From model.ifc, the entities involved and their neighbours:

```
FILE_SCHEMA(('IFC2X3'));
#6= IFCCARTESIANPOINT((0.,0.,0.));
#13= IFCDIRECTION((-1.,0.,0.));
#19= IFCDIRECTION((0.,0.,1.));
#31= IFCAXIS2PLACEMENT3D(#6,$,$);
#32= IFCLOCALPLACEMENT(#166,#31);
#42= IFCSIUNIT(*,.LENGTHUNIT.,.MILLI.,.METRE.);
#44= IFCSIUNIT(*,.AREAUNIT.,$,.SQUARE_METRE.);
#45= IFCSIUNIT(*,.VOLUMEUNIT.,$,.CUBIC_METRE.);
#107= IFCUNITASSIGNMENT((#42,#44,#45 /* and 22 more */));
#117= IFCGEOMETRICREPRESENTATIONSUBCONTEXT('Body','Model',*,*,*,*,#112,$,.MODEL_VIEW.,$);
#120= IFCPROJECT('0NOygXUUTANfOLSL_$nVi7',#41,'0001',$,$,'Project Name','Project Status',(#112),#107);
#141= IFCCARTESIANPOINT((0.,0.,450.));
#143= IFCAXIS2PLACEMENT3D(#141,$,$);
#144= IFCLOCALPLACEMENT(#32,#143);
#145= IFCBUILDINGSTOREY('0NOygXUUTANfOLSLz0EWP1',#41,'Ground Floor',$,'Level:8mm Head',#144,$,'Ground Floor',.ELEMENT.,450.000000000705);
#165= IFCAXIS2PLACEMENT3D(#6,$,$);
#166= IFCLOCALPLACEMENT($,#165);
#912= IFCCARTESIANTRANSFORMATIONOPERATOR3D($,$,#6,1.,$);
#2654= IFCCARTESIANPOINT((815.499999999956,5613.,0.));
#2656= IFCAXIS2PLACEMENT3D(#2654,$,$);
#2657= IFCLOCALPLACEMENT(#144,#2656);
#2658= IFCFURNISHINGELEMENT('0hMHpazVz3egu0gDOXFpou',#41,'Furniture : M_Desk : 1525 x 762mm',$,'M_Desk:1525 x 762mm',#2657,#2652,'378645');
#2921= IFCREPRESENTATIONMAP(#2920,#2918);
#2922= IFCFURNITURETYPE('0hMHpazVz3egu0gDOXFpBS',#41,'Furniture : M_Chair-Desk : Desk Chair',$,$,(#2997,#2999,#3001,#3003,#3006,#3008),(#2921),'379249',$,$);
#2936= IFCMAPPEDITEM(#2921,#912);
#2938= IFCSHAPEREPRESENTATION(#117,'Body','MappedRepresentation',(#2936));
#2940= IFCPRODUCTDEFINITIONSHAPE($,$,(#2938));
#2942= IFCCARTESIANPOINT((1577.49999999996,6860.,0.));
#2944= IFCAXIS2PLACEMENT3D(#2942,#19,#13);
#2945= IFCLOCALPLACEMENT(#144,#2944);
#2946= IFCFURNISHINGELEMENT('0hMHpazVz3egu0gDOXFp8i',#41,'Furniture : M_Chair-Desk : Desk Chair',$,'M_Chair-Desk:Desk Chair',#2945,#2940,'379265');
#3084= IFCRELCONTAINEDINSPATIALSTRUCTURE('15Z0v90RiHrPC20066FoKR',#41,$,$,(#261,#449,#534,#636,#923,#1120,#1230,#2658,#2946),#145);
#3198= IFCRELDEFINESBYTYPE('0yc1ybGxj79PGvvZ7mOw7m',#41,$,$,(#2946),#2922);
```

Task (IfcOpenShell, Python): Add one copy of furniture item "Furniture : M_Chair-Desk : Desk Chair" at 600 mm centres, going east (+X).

```python
import numpy as np
import ifcopenshell
import ifcopenshell.api.geometry
import ifcopenshell.api.root
import ifcopenshell.util.element
import ifcopenshell.util.placement

model = ifcopenshell.open("model.ifc")


def reuse_history(source, copy):
    """copy_class also copies each property set's owner history, people and application; keep the originals."""
    for rel in copy.IsDefinedBy:
        if rel.is_a("IfcRelDefinesByProperties") and (history := rel.RelatingPropertyDefinition.OwnerHistory):
            rel.RelatingPropertyDefinition.OwnerHistory = source.OwnerHistory
            ifcopenshell.util.element.remove_deep2(model, history)


source = model.by_guid("0hMHpazVz3egu0gDOXFp8i")
base = ifcopenshell.util.placement.get_local_placement(source.ObjectPlacement)
step = np.array([1.0, 0.0, 0.0]) * 600.0

for i in range(1, 2):
    copy = ifcopenshell.api.root.copy_class(model, product=source)
    copy.Representation = ifcopenshell.util.element.copy_deep(
        model, source.Representation, exclude=["IfcGeometricRepresentationContext", "IfcRepresentationMap"]
    )
    copy.Tag = None
    reuse_history(source, copy)
    matrix = base.copy()
    matrix[:3, 3] += i * step
    print("added at", matrix[:3, 3].round(3) + 0.0)
    ifcopenshell.api.geometry.edit_object_placement(model, product=copy, matrix=matrix, is_si=False)

model.write("model_edited.ifc")
```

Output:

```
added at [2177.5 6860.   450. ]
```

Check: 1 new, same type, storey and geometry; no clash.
